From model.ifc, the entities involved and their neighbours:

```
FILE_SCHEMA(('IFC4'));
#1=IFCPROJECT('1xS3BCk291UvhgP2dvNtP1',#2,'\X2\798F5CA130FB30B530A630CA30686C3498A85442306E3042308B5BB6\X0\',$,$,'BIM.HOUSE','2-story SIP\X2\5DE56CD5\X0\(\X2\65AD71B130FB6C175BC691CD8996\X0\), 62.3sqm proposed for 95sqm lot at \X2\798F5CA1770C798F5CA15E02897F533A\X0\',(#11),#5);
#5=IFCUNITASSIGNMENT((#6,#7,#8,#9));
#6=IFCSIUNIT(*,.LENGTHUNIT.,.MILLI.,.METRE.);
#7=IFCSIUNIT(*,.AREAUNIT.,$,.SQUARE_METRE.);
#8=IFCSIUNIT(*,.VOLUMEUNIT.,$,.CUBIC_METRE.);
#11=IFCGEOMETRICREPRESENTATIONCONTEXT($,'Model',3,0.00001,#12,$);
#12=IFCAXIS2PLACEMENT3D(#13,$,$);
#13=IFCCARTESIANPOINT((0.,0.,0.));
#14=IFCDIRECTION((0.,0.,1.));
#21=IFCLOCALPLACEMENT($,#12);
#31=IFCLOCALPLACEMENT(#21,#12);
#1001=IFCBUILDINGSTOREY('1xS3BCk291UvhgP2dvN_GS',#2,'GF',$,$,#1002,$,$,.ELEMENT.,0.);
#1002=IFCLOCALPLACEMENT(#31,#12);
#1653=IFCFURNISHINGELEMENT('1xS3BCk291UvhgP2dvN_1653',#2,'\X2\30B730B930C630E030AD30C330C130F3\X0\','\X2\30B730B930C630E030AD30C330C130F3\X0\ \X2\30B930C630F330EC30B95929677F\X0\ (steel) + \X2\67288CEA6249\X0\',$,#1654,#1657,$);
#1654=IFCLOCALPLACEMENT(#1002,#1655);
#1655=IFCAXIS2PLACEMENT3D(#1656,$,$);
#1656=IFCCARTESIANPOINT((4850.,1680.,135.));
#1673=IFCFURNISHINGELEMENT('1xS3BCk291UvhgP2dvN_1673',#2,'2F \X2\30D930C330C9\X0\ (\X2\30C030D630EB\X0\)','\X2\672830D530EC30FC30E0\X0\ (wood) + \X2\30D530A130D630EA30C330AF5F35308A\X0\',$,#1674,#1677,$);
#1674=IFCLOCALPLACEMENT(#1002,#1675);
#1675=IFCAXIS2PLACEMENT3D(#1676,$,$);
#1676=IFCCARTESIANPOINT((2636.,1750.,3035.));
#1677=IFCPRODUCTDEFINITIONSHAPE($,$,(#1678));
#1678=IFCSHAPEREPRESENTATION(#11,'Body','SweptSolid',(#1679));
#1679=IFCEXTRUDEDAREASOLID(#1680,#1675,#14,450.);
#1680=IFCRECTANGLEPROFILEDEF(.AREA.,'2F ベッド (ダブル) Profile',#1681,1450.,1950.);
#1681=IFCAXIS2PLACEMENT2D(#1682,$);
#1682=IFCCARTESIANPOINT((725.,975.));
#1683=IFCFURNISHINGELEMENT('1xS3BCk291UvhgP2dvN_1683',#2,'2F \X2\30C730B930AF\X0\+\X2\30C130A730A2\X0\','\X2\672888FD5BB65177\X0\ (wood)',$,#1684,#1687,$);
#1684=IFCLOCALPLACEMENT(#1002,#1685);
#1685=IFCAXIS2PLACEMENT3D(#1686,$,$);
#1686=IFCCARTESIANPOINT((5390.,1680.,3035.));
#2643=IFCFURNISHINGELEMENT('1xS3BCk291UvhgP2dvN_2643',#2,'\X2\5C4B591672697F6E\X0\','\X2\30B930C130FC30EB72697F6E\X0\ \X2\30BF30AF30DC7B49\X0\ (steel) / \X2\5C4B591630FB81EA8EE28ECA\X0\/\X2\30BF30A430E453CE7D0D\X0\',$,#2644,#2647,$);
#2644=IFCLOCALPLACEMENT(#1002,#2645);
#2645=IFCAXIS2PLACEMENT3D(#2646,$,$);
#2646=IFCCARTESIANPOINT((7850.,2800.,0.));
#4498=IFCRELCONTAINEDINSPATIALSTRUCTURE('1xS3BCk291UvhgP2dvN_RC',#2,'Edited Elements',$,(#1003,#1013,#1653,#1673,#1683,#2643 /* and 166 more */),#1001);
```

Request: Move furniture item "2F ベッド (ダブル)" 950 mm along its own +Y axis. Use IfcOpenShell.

```python
import ifcopenshell
import ifcopenshell.api.geometry
import ifcopenshell.util.placement

model = ifcopenshell.open("model.ifc")

item = model.by_guid("1xS3BCk291UvhgP2dvN_1673")
matrix = ifcopenshell.util.placement.get_local_placement(item.ObjectPlacement)
matrix[:3, 3] += matrix[:3, 1] * 950.0
ifcopenshell.api.geometry.edit_object_placement(model, product=item, matrix=matrix, is_si=False)

print(ifcopenshell.util.placement.get_local_placement(item.ObjectPlacement).round(3) + 0.0)

model.write("model_updated.ifc")
```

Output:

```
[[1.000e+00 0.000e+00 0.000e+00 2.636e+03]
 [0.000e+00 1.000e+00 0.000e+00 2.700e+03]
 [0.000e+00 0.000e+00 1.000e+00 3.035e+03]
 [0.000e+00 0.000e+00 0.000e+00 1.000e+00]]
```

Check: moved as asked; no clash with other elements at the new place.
